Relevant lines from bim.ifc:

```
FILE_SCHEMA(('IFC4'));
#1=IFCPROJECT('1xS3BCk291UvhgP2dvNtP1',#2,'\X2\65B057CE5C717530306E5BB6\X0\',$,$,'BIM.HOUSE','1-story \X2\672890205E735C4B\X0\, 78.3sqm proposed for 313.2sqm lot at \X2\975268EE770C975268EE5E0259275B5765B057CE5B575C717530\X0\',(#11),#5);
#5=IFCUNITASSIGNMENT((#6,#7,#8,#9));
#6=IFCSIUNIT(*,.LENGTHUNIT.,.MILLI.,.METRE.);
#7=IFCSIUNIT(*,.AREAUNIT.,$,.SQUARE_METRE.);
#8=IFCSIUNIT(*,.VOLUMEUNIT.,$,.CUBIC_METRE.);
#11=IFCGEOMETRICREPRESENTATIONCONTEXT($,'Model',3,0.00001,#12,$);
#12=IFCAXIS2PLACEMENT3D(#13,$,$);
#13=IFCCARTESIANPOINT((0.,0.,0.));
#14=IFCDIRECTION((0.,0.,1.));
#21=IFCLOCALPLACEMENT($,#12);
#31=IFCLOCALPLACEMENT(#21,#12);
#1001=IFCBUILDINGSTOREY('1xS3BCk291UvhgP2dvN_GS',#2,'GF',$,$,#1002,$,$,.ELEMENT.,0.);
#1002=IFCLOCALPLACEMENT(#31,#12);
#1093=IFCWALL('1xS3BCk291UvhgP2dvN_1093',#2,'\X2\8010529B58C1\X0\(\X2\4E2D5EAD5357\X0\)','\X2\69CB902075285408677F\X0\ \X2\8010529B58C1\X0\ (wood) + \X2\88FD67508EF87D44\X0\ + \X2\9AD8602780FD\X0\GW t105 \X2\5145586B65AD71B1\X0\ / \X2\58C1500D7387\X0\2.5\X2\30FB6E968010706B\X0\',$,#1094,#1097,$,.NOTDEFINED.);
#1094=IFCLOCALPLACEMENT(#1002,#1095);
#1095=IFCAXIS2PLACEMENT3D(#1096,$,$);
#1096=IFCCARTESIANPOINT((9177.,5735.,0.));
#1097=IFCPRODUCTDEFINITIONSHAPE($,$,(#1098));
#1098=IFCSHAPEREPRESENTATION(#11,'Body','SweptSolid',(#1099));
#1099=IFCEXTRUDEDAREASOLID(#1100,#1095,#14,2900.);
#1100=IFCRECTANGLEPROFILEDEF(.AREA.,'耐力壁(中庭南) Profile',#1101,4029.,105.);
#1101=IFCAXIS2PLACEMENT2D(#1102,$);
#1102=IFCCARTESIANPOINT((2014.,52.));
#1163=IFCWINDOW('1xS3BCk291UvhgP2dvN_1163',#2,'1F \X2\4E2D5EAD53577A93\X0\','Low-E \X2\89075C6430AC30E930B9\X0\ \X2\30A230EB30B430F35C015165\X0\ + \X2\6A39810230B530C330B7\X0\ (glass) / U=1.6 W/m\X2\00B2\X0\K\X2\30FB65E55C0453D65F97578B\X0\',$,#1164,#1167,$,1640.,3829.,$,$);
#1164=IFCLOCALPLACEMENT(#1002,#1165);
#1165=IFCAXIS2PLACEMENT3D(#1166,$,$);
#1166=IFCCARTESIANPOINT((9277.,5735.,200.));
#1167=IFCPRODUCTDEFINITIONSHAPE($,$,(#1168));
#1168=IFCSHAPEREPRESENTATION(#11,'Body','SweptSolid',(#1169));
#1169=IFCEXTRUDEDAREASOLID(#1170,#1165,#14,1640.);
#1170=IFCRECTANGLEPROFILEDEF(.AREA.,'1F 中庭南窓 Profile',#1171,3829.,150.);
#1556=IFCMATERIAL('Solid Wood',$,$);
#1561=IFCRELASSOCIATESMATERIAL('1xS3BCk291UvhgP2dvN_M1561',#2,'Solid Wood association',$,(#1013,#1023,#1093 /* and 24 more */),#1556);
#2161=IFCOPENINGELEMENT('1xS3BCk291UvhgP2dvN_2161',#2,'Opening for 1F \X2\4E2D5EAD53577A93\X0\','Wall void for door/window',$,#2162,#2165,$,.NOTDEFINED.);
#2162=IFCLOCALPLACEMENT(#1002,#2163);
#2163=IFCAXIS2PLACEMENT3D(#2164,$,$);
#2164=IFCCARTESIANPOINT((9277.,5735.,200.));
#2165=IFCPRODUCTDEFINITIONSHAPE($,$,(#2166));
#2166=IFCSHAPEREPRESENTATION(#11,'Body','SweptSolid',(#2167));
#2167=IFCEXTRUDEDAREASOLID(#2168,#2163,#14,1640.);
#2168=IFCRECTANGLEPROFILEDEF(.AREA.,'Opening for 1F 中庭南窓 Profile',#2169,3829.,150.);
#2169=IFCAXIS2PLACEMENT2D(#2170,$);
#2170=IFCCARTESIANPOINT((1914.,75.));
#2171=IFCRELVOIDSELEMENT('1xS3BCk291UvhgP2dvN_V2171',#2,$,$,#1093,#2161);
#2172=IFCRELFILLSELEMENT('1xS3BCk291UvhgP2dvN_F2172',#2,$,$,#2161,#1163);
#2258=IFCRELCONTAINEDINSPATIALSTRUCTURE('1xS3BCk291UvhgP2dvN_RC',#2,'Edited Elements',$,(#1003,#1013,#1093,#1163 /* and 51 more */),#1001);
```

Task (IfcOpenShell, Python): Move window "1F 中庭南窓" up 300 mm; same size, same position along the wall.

```python
import numpy as np
import ifcopenshell
import ifcopenshell.api.geometry
import ifcopenshell.util.placement
import ifcopenshell.util.unit

model = ifcopenshell.open("bim.ifc")
unit_scale = ifcopenshell.util.unit.calculate_unit_scale(model)

window = model.by_guid("1xS3BCk291UvhgP2dvN_1163")
opening = window.FillsVoids[0].RelatingOpeningElement
dz = 300.0

shift = np.array([0.0, 0.0, dz])
# The window is not placed relative to its opening, so move both.
for product in (opening, window):
    matrix = ifcopenshell.util.placement.get_local_placement(product.ObjectPlacement)
    matrix[:3, 3] += shift
    ifcopenshell.api.geometry.edit_object_placement(model, product=product, matrix=matrix, is_si=False)

print(f"moved by {dz * unit_scale:+.3f} m")

model.write("bim_updated.ifc")
```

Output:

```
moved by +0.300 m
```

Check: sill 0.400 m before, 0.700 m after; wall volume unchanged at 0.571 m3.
